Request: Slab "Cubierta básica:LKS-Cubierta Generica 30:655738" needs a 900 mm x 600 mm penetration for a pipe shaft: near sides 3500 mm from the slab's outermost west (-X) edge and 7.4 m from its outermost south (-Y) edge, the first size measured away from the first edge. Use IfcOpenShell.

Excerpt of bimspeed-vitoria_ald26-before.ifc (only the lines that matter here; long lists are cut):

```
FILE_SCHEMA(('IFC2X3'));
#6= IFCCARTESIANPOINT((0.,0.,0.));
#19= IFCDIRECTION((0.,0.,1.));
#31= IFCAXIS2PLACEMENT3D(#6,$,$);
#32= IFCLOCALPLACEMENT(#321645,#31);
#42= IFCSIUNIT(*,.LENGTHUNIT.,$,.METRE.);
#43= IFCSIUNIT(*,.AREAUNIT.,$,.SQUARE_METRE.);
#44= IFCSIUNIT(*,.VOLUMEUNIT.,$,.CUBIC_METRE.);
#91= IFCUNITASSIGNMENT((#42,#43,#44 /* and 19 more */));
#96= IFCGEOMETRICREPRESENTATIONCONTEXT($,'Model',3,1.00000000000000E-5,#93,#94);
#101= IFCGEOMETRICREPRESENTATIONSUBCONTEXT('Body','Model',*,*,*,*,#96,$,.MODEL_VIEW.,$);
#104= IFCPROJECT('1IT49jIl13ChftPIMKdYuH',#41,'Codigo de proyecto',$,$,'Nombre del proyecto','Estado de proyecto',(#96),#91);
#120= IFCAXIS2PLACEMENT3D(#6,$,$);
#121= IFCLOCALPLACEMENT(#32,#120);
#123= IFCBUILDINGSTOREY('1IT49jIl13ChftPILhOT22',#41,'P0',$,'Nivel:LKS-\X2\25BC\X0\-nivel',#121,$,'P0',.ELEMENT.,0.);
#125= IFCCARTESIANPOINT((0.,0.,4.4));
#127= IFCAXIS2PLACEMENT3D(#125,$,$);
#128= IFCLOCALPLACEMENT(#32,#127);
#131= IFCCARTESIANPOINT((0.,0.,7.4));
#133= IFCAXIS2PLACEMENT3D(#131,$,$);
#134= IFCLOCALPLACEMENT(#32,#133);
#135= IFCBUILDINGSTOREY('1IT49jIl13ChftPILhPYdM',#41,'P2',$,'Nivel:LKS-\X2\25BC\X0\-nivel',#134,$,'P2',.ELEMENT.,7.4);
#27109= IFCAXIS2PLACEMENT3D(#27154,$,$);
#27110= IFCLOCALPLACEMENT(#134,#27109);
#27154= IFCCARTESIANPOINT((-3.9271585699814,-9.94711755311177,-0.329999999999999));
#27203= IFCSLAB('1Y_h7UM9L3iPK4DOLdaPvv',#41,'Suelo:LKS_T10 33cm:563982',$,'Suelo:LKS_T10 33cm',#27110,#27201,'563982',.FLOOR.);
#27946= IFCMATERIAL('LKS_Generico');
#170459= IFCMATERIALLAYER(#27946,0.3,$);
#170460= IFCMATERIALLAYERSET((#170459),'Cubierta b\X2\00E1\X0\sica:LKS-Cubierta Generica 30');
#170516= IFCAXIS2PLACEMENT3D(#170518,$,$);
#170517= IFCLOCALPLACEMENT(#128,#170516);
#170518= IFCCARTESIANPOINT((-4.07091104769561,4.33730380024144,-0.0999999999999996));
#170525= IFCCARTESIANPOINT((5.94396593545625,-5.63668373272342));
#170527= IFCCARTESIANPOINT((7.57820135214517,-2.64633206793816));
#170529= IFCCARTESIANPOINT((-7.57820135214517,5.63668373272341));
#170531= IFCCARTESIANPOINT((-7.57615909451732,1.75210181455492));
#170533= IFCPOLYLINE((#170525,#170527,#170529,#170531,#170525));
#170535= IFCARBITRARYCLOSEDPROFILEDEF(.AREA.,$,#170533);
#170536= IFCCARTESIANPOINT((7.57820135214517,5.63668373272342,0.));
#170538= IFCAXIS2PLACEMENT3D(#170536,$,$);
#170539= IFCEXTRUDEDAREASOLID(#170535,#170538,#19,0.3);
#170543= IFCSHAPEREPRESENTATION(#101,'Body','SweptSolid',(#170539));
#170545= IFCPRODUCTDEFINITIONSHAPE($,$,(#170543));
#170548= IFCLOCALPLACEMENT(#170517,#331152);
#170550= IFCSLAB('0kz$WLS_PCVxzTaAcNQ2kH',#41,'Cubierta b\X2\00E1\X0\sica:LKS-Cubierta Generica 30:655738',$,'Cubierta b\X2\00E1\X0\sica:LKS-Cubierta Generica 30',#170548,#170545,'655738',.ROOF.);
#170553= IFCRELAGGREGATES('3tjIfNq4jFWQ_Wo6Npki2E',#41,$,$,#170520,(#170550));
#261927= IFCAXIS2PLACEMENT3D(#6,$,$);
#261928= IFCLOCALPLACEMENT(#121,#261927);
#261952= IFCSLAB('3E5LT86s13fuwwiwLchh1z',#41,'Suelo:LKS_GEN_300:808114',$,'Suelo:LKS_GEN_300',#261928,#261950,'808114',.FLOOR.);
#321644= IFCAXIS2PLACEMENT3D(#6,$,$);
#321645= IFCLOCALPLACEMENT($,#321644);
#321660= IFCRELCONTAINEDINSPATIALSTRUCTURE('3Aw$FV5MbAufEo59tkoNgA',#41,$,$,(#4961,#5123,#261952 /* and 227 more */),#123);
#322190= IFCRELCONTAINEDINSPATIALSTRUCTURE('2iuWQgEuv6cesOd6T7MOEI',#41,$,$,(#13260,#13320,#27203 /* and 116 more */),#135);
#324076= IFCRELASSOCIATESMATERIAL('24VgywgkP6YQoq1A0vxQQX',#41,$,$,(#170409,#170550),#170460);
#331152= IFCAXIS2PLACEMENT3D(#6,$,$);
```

```python
import numpy as np
import ifcopenshell
import ifcopenshell.api.feature
import ifcopenshell.api.geometry
import ifcopenshell.api.root
import ifcopenshell.geom
import ifcopenshell.util.placement
import ifcopenshell.util.representation
import ifcopenshell.util.shape
import ifcopenshell.util.unit

model = ifcopenshell.open("bimspeed-vitoria_ald26-before.ifc")
unit_scale = ifcopenshell.util.unit.calculate_unit_scale(model)
settings = ifcopenshell.geom.settings()


def volume(element):
    """Net volume in cubic metres, openings subtracted."""
    shape = ifcopenshell.geom.create_shape(settings, element)
    return ifcopenshell.util.shape.get_volume(shape.geometry)


slab = model.by_guid("0kz$WLS_PCVxzTaAcNQ2kH")
before = volume(slab)

# Extent in the slab's own axes, in metres. The edges named are its -X and -Y sides.
slab_shape = ifcopenshell.geom.create_shape(settings, slab)
vertices = ifcopenshell.util.shape.get_vertices(slab_shape.geometry)
x_min, y_min, bottom = vertices.min(axis=0)
top = vertices[:, 2].max()

opening = ifcopenshell.api.root.create_entity(model, ifc_class="IfcOpeningElement", name="Pipe shaft opening")
context = ifcopenshell.util.representation.get_context(model, "Model", "Body", "MODEL_VIEW")
width, depth = 0.9, 0.6
outline = [(0.0, 0.0), (width, 0.0), (width, depth), (0.0, depth), (0.0, 0.0)]
# Overshoot both faces by 50 mm so the cut is clean.
shape = ifcopenshell.api.geometry.add_slab_representation(
    model, context=context, depth=top - bottom + 0.1, polyline=outline
)
ifcopenshell.api.geometry.assign_representation(model, product=opening, representation=shape)

matrix = ifcopenshell.util.placement.get_local_placement(slab.ObjectPlacement)
matrix[:, 3] = matrix @ np.append(np.array([x_min + 3.5, y_min + 7.4, bottom - 0.05]) / unit_scale, 1.0)
ifcopenshell.api.geometry.edit_object_placement(model, product=opening, matrix=matrix, is_si=False)
ifcopenshell.api.feature.add_feature(model, feature=opening, element=slab)

after = volume(slab)

print(f"slab volume {before:.3f} -> {after:.3f} m3")

model.write("bimspeed-vitoria_ald26-before_edited.ifc")
```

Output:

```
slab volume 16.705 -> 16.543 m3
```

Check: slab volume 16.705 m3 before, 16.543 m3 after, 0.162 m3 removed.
